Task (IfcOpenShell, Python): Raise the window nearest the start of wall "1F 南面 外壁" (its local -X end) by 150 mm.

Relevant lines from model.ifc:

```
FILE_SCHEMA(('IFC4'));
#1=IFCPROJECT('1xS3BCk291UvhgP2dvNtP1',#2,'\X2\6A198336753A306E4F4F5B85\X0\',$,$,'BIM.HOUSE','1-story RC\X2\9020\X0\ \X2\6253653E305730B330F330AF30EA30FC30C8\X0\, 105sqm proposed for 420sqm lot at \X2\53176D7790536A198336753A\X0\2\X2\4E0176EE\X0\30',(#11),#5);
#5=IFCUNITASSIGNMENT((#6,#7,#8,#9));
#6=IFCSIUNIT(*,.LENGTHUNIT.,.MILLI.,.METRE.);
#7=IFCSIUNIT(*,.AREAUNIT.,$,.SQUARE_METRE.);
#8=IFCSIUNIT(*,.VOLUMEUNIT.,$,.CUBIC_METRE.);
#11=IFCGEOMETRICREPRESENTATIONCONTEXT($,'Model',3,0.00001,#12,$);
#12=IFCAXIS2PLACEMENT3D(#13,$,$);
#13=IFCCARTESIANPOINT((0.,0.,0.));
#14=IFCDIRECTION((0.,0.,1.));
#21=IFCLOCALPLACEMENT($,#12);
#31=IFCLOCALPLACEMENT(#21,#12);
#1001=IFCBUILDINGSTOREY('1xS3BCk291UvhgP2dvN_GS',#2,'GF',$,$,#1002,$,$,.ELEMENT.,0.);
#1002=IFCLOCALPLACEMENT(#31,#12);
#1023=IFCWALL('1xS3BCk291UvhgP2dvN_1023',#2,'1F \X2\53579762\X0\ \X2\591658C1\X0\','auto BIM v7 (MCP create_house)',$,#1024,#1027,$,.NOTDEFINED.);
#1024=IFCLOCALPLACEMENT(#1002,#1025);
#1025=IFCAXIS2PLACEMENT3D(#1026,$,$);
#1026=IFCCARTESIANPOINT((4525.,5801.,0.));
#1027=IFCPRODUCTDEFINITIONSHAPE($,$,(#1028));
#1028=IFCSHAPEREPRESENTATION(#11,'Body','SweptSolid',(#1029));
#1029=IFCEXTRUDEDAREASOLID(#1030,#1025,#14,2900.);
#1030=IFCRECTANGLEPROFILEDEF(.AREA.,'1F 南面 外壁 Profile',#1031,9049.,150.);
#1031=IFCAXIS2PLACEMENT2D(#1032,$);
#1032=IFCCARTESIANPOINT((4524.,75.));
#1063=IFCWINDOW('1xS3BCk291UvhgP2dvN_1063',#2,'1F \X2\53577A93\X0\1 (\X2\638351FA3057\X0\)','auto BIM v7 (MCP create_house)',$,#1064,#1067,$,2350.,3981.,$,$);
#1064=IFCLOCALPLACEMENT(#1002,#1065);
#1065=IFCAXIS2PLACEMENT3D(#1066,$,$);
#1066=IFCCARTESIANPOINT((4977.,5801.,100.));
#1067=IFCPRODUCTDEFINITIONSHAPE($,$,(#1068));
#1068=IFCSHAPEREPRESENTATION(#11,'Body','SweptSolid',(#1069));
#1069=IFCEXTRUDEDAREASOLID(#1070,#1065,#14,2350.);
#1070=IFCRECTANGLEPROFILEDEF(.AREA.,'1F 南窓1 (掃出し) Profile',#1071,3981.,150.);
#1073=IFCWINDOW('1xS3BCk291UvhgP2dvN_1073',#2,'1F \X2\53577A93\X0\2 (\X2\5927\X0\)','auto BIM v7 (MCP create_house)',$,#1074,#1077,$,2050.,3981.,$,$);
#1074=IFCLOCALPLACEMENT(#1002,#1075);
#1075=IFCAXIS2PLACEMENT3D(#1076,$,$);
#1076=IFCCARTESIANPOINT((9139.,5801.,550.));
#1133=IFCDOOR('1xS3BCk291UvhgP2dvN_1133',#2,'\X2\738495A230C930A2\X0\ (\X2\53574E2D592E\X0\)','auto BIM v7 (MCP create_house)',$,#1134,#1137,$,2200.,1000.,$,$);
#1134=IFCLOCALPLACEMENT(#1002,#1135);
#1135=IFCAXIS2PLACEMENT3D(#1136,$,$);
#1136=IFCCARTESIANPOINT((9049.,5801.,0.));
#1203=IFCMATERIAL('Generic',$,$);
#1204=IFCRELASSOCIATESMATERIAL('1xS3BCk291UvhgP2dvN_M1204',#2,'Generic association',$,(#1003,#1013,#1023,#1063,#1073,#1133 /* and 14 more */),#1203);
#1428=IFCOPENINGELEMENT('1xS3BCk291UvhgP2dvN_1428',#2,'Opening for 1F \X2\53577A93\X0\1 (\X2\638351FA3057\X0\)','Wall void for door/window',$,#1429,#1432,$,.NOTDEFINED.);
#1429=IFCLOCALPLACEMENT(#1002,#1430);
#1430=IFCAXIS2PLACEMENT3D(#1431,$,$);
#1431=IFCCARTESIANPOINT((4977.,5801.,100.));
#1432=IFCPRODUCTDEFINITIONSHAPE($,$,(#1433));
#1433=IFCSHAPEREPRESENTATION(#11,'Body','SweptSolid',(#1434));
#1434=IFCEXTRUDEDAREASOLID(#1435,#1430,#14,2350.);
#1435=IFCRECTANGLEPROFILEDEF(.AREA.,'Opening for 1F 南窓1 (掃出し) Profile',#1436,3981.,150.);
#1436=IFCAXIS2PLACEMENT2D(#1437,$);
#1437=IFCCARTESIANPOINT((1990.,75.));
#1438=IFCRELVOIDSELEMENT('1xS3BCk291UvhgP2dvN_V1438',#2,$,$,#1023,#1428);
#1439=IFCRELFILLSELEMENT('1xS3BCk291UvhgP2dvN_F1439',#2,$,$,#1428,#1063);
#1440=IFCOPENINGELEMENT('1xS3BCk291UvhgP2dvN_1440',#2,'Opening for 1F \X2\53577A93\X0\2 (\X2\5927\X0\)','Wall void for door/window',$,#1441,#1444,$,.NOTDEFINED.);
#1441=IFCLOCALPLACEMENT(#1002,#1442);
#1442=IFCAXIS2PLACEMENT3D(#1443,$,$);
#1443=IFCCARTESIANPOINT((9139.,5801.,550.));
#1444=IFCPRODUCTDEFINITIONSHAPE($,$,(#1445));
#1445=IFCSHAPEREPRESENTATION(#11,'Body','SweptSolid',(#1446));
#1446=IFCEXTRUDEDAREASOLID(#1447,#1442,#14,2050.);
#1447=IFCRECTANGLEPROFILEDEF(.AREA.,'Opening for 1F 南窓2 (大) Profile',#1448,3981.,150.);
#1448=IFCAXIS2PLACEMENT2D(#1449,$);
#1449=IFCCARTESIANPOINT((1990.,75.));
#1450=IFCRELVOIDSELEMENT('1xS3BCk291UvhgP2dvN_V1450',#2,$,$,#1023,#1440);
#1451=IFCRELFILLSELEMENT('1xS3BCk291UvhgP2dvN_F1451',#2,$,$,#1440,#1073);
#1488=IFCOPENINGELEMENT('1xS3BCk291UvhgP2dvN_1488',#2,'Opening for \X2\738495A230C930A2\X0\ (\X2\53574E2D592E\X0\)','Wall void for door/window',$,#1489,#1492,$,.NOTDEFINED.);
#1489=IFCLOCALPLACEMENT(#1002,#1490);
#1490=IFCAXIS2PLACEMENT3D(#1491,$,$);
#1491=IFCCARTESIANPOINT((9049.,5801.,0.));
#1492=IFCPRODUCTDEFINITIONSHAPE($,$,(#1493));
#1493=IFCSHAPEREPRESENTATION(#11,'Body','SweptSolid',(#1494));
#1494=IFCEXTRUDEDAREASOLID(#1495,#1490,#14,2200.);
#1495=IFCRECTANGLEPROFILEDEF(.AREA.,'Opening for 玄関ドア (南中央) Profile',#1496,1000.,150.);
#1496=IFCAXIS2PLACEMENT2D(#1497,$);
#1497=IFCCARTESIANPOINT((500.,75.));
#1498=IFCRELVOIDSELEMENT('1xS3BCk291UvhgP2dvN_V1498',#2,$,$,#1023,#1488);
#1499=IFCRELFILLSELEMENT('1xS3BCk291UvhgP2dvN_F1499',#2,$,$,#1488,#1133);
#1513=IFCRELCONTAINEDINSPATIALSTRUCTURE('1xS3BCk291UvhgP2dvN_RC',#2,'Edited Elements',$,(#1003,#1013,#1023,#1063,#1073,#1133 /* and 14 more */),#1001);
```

```python
import numpy as np
import ifcopenshell
import ifcopenshell.api.geometry
import ifcopenshell.util.placement
import ifcopenshell.util.unit

model = ifcopenshell.open("model.ifc")
unit_scale = ifcopenshell.util.unit.calculate_unit_scale(model)

window = model.by_id(1063)
opening = window.FillsVoids[0].RelatingOpeningElement
dz = 0.15 / unit_scale

shift = np.array([0.0, 0.0, dz])
# The window is not placed relative to its opening, so move both.
for product in (opening, window):
    matrix = ifcopenshell.util.placement.get_local_placement(product.ObjectPlacement)
    matrix[:3, 3] += shift
    ifcopenshell.api.geometry.edit_object_placement(model, product=product, matrix=matrix, is_si=False)

print(f"moved by {dz * unit_scale:+.3f} m")

model.write("model_edited.ifc")
```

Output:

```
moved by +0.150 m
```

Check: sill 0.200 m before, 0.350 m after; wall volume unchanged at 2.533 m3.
